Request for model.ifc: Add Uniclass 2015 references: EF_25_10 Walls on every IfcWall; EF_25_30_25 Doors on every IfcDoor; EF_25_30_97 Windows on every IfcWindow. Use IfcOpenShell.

First a look at what the model holds.

```python
import ifcopenshell

model = ifcopenshell.open("model.ifc")
print(model.schema)
print("classifications:", [c.Name for c in model.by_type("IfcClassification")])
for ifc_class in ("IfcDoor", "IfcRoof", "IfcStair", "IfcWall", "IfcWindow"):
    print(ifc_class, len(model.by_type(ifc_class)))
```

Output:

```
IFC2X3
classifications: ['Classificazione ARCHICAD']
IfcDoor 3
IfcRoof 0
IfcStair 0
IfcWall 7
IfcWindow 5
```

```python
import ifcopenshell
import ifcopenshell.api.classification

model = ifcopenshell.open("model.ifc")

# IFC2X3 requires Source and Edition and has no link from the project to the system.
system = model.create_entity("IfcClassification", Source="NBS", Edition="2015", Name="Uniclass 2015")

codes = {
    "IfcWall": ("EF_25_10", "Walls"),
    "IfcDoor": ("EF_25_30_25", "Doors"),
    "IfcWindow": ("EF_25_30_97", "Windows"),
}
for ifc_class, (code, name) in codes.items():
    products = model.by_type(ifc_class)
    ifcopenshell.api.classification.add_reference(
        model, products=products, classification=system, identification=code, name=name
    )
    print(code, len(products))

model.write("model_rev.ifc")
```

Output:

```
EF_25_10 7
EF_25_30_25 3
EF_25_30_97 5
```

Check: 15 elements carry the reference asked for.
